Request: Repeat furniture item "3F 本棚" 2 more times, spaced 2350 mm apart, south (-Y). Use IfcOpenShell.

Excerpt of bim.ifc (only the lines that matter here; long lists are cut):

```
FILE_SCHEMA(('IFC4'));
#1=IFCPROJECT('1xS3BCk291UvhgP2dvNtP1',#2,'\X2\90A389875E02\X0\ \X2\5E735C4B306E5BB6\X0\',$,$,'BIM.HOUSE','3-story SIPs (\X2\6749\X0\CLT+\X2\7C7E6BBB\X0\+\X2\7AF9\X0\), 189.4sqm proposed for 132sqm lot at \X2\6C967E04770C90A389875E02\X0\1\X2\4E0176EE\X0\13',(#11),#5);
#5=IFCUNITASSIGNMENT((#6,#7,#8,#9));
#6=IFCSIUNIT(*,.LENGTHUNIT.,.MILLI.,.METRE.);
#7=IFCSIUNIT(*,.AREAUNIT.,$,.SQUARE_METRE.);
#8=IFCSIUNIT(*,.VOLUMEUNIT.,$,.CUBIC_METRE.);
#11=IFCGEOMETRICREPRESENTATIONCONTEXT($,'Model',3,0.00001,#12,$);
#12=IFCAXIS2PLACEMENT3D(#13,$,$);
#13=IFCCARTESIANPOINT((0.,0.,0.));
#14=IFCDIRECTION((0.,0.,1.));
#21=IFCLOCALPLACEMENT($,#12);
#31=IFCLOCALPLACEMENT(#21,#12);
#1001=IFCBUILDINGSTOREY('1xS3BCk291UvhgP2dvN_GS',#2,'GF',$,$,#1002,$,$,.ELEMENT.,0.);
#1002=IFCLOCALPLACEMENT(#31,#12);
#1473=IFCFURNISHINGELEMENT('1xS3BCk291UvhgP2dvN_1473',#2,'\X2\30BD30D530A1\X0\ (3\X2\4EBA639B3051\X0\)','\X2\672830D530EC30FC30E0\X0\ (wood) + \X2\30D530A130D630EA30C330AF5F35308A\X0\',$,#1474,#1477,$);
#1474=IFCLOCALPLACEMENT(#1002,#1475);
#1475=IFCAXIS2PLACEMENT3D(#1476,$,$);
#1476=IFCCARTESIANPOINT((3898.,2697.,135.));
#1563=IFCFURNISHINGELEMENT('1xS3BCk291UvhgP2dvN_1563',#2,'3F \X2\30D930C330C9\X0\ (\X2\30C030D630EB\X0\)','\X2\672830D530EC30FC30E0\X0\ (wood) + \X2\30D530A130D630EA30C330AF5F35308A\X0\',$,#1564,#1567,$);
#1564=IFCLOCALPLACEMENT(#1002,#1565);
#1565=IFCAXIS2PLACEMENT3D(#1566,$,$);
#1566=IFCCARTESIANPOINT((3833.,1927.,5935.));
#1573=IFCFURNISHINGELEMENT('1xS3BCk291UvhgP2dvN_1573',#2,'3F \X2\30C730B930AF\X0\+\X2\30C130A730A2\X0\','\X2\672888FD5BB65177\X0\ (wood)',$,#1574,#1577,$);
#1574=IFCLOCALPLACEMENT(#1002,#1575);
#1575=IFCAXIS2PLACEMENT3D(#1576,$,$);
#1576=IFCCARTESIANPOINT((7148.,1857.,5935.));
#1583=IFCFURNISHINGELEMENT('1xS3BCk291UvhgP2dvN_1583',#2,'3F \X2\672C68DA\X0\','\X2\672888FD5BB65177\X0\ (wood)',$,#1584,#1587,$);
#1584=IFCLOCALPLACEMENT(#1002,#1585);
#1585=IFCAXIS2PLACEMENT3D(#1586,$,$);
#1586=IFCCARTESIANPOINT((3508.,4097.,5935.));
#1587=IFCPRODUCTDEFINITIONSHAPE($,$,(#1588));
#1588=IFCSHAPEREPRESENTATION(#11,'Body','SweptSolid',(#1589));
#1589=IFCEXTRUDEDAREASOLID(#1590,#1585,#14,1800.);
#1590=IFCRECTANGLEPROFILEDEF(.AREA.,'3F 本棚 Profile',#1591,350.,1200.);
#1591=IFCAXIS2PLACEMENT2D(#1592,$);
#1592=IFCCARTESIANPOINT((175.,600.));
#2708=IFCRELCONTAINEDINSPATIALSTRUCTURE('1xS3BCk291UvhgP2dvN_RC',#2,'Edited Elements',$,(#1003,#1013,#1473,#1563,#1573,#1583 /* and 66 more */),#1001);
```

```python
import numpy as np
import ifcopenshell
import ifcopenshell.api.geometry
import ifcopenshell.api.root
import ifcopenshell.util.element
import ifcopenshell.util.placement

model = ifcopenshell.open("bim.ifc")


def reuse_history(source, copy):
    """copy_class also copies each property set's owner history, people and application; keep the originals."""
    for rel in copy.IsDefinedBy:
        if rel.is_a("IfcRelDefinesByProperties") and (history := rel.RelatingPropertyDefinition.OwnerHistory):
            rel.RelatingPropertyDefinition.OwnerHistory = source.OwnerHistory
            ifcopenshell.util.element.remove_deep2(model, history)


source = model.by_guid("1xS3BCk291UvhgP2dvN_1583")
base = ifcopenshell.util.placement.get_local_placement(source.ObjectPlacement)
step = np.array([0.0, -1.0, 0.0]) * 2350.0

for i in range(1, 3):
    copy = ifcopenshell.api.root.copy_class(model, product=source)
    copy.Representation = ifcopenshell.util.element.copy_deep(
        model, source.Representation, exclude=["IfcGeometricRepresentationContext", "IfcRepresentationMap"]
    )
    reuse_history(source, copy)
    matrix = base.copy()
    matrix[:3, 3] += i * step
    print("added at", matrix[:3, 3].round(3) + 0.0)
    ifcopenshell.api.geometry.edit_object_placement(model, product=copy, matrix=matrix, is_si=False)

model.write("bim_v2.ifc")
```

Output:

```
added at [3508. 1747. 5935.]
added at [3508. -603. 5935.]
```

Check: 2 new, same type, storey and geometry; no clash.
